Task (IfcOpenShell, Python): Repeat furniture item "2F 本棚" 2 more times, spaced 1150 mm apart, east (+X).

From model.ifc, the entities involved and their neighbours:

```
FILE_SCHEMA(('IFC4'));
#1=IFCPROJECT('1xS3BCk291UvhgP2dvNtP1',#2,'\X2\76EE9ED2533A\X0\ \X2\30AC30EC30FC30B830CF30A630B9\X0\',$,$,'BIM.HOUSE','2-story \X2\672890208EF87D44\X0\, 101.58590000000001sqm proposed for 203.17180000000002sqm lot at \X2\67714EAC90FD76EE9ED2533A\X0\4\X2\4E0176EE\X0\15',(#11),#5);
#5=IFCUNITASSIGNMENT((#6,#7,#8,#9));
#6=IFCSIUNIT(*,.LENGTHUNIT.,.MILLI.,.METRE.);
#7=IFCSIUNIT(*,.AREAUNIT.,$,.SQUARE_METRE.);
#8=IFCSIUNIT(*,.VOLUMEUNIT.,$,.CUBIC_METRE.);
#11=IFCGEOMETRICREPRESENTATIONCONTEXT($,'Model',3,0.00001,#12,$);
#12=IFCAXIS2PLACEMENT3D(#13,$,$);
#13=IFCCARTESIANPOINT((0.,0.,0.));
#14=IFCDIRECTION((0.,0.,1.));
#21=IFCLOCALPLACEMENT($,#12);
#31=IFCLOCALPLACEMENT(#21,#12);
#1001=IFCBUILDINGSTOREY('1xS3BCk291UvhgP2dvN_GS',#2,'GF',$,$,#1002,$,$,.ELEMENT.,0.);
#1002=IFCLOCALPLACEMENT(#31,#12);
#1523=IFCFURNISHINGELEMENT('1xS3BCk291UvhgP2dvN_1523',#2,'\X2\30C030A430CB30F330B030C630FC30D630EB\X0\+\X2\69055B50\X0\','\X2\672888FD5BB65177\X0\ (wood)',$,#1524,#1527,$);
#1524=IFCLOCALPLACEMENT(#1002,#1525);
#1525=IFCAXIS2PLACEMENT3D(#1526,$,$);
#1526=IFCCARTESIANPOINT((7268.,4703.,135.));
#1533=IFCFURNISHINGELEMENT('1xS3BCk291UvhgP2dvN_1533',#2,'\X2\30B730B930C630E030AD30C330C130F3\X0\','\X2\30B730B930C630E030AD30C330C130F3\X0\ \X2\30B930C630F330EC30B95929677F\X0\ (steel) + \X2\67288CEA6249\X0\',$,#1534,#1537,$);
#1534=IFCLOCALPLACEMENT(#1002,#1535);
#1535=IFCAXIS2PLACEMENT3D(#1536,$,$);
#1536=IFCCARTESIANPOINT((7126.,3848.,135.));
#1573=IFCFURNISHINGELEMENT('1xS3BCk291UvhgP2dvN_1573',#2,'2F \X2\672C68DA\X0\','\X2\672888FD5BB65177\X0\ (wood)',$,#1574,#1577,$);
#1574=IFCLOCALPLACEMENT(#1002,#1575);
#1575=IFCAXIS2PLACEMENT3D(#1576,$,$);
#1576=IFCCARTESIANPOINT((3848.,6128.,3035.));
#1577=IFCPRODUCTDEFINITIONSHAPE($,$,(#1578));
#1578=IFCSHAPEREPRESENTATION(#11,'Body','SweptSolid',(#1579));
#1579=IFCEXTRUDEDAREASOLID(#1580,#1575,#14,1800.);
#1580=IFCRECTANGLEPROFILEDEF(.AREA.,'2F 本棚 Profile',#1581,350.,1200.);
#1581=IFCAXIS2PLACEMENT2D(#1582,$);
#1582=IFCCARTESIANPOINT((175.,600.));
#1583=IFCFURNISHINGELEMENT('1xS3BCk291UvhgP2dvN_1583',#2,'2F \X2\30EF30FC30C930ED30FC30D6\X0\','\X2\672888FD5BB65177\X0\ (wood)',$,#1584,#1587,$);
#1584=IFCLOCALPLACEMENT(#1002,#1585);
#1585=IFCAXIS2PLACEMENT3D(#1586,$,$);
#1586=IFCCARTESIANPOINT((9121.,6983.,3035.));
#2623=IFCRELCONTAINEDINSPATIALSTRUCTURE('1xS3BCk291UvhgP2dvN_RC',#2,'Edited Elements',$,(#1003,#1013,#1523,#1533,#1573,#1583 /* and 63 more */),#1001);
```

```python
import numpy as np
import ifcopenshell
import ifcopenshell.api.geometry
import ifcopenshell.api.root
import ifcopenshell.util.element
import ifcopenshell.util.placement
import ifcopenshell.util.unit

model = ifcopenshell.open("model.ifc")
unit_scale = ifcopenshell.util.unit.calculate_unit_scale(model)


def reuse_history(source, copy):
    """copy_class also copies each property set's owner history, people and application; keep the originals."""
    for rel in copy.IsDefinedBy:
        if rel.is_a("IfcRelDefinesByProperties") and (history := rel.RelatingPropertyDefinition.OwnerHistory):
            rel.RelatingPropertyDefinition.OwnerHistory = source.OwnerHistory
            ifcopenshell.util.element.remove_deep2(model, history)


source = model.by_guid("1xS3BCk291UvhgP2dvN_1573")
base = ifcopenshell.util.placement.get_local_placement(source.ObjectPlacement)
step = np.array([1.0, 0.0, 0.0]) * 1.15 / unit_scale

for i in range(1, 3):
    copy = ifcopenshell.api.root.copy_class(model, product=source)
    copy.Representation = ifcopenshell.util.element.copy_deep(
        model, source.Representation, exclude=["IfcGeometricRepresentationContext", "IfcRepresentationMap"]
    )
    reuse_history(source, copy)
    matrix = base.copy()
    matrix[:3, 3] += i * step
    print("added at", matrix[:3, 3].round(3) + 0.0)
    ifcopenshell.api.geometry.edit_object_placement(model, product=copy, matrix=matrix, is_si=False)

model.write("model_edited.ifc")
```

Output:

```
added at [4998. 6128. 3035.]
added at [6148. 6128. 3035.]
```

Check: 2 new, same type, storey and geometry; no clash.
